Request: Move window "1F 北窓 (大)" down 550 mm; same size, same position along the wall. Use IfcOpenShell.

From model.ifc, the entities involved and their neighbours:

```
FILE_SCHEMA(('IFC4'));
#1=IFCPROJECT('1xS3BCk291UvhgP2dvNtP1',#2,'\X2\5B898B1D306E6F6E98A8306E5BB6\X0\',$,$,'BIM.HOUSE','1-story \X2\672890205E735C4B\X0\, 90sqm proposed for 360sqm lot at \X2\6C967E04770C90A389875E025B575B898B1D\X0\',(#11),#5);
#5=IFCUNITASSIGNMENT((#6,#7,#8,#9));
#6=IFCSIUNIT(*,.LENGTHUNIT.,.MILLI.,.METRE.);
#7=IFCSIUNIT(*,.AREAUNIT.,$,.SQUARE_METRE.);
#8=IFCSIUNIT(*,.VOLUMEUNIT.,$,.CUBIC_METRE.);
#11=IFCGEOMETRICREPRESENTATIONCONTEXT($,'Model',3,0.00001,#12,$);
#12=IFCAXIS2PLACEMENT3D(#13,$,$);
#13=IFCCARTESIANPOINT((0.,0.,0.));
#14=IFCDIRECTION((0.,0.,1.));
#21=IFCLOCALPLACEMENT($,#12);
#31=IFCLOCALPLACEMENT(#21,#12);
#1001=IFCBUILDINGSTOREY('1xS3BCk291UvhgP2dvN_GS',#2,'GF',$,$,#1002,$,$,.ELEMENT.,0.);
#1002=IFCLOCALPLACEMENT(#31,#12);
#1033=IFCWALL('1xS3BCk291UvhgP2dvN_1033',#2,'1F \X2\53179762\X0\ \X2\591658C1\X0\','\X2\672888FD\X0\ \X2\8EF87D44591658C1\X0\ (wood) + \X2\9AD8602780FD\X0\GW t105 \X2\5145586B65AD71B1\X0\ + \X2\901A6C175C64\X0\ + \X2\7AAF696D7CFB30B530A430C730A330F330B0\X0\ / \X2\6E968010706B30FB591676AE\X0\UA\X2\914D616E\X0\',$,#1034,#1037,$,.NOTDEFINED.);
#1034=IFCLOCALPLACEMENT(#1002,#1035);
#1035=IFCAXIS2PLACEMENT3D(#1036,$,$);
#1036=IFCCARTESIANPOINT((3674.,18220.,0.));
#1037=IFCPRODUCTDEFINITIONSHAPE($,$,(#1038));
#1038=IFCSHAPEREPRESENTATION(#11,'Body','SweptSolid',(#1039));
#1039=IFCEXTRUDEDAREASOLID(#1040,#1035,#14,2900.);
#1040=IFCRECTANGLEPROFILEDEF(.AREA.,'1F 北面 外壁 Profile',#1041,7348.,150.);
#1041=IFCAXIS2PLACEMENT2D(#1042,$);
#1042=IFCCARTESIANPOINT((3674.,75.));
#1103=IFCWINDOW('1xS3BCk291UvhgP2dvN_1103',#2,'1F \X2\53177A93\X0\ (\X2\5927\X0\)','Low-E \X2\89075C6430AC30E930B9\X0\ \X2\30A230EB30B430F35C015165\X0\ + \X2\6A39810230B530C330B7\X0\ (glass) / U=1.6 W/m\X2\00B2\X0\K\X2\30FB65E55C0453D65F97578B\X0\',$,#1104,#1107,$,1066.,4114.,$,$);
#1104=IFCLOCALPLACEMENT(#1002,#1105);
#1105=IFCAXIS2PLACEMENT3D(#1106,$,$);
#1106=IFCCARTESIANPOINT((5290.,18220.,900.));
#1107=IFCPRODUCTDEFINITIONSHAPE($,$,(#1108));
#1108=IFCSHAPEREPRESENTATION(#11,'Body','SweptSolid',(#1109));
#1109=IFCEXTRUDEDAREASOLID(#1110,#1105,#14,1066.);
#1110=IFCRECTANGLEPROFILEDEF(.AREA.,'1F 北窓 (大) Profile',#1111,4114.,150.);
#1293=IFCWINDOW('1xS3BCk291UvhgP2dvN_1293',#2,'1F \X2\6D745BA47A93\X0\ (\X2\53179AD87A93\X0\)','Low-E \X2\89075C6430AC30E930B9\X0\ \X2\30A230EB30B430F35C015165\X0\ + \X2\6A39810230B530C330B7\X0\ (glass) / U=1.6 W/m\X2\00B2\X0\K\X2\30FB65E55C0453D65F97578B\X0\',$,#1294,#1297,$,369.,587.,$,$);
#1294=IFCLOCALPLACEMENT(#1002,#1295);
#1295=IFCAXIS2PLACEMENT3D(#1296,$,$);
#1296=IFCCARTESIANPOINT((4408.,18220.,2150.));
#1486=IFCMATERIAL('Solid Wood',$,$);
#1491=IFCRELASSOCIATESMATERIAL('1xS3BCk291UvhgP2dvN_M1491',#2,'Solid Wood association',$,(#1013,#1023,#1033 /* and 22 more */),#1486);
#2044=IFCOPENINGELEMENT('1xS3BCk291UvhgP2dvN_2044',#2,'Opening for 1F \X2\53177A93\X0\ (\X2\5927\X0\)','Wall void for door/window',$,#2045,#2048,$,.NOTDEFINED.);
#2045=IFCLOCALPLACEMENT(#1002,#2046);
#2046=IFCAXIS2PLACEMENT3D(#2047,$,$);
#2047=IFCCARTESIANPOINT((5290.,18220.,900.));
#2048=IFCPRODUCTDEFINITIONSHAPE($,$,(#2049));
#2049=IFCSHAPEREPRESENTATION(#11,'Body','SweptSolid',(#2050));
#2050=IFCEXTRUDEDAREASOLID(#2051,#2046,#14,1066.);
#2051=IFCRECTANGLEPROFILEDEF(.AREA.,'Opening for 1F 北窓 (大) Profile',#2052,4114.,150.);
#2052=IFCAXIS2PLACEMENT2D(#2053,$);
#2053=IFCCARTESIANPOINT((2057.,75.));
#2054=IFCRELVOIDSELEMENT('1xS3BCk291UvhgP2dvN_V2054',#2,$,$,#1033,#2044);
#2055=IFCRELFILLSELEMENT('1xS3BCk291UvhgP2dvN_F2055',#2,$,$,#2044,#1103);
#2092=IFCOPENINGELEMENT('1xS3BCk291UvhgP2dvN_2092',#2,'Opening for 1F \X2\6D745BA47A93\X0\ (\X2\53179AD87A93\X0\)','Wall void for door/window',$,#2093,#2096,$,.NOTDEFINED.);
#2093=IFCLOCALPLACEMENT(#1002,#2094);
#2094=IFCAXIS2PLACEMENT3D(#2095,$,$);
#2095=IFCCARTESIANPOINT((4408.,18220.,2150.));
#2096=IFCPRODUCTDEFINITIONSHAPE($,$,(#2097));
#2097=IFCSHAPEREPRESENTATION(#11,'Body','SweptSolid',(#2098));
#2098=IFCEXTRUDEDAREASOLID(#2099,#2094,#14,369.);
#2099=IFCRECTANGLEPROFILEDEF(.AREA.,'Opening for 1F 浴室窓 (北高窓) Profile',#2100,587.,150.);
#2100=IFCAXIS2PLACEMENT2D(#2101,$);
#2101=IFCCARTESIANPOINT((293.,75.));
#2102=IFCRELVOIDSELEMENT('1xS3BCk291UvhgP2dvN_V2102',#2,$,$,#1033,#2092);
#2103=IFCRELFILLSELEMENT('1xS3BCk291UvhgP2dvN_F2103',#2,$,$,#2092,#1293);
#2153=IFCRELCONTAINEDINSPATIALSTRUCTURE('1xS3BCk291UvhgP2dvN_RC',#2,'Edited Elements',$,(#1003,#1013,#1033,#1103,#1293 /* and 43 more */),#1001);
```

```python
import numpy as np
import ifcopenshell
import ifcopenshell.api.geometry
import ifcopenshell.util.placement
import ifcopenshell.util.unit

model = ifcopenshell.open("model.ifc")
unit_scale = ifcopenshell.util.unit.calculate_unit_scale(model)

window = model.by_guid("1xS3BCk291UvhgP2dvN_1103")
opening = window.FillsVoids[0].RelatingOpeningElement
dz = -0.55 / unit_scale

shift = np.array([0.0, 0.0, dz])
# The window is not placed relative to its opening, so move both.
for product in (opening, window):
    matrix = ifcopenshell.util.placement.get_local_placement(product.ObjectPlacement)
    matrix[:3, 3] += shift
    ifcopenshell.api.geometry.edit_object_placement(model, product=product, matrix=matrix, is_si=False)

print(f"moved by {dz * unit_scale:+.3f} m")

model.write("model_v2.ifc")
```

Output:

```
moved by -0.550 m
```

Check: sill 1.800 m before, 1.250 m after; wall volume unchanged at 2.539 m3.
